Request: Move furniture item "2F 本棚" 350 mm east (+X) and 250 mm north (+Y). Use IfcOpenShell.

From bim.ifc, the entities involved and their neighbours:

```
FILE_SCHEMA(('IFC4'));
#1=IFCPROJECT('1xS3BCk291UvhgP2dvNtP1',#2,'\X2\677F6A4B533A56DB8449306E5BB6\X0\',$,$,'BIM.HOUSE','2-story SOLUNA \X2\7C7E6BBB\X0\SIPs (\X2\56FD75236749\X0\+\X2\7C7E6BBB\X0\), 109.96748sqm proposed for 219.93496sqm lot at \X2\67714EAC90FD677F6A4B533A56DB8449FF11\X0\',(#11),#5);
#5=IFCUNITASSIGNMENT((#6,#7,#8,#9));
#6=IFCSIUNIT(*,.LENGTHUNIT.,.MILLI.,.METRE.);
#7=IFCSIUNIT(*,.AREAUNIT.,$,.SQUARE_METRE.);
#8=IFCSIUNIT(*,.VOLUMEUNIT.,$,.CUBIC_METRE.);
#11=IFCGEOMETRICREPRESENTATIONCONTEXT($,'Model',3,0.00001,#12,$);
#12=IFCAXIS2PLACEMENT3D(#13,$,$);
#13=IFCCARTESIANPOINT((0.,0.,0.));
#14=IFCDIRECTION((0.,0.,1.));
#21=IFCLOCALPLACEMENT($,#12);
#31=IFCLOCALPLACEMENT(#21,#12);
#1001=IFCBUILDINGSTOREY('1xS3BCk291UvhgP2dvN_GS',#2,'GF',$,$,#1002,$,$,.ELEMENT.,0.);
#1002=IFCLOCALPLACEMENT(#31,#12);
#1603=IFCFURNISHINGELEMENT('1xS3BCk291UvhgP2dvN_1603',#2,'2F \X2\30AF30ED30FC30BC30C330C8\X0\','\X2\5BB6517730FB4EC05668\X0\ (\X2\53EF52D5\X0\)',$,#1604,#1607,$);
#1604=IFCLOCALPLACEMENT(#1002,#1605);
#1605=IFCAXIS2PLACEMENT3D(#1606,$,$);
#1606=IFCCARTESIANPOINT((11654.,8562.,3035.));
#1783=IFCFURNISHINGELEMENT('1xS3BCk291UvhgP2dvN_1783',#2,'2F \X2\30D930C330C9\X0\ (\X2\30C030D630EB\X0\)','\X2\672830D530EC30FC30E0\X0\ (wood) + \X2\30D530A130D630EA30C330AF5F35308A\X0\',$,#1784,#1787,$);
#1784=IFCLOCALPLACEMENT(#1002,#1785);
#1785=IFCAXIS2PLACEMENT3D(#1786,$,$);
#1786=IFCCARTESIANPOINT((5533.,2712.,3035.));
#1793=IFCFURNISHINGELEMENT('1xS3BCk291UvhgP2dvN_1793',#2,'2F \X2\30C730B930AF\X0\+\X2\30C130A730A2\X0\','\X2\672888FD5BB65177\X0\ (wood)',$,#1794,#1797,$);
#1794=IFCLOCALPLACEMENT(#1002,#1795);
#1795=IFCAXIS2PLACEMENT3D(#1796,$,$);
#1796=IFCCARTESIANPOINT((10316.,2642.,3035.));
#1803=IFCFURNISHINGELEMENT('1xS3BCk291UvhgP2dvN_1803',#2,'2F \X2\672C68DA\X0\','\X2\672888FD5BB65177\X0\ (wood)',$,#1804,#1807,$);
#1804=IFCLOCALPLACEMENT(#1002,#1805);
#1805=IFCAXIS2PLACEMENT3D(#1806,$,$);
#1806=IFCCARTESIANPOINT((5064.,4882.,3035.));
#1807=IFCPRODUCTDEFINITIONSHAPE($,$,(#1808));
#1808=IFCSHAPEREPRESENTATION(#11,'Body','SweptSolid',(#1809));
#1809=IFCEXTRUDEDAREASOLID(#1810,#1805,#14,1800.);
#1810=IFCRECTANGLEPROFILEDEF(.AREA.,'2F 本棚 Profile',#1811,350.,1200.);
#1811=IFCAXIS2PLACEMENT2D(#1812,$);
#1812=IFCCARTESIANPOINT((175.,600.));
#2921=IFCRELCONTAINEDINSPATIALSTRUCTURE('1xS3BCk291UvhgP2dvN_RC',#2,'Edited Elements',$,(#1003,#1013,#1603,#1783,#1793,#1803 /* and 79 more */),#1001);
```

```python
import ifcopenshell
import ifcopenshell.api.geometry
import ifcopenshell.util.placement
import ifcopenshell.util.unit

model = ifcopenshell.open("bim.ifc")
unit_scale = ifcopenshell.util.unit.calculate_unit_scale(model)

item = model.by_guid("1xS3BCk291UvhgP2dvN_1803")
matrix = ifcopenshell.util.placement.get_local_placement(item.ObjectPlacement)
matrix[0, 3] += 0.35 / unit_scale
matrix[1, 3] += 0.25 / unit_scale
ifcopenshell.api.geometry.edit_object_placement(model, product=item, matrix=matrix, is_si=False)

print(ifcopenshell.util.placement.get_local_placement(item.ObjectPlacement).round(3) + 0.0)

model.write("bim_rev.ifc")
```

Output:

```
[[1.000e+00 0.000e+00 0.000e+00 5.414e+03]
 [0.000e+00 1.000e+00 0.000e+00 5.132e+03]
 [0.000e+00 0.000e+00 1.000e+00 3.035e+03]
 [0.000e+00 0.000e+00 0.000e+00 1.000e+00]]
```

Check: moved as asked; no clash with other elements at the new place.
